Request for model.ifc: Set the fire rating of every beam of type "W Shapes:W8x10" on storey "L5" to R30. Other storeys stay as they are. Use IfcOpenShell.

First a look at what the model holds.

```python
import ifcopenshell
import ifcopenshell.util.element

model = ifcopenshell.open("model.ifc")
print(model.schema)
storey = next(s for s in model.by_type("IfcBuildingStorey") if s.Name == "L5")
beams = [e for e in ifcopenshell.util.element.get_decomposition(storey) if e.is_a("IfcBeam")]
seen = {}
for e in beams:
    element_type = ifcopenshell.util.element.get_type(e)
    key = (element_type.Name if element_type != e and element_type else None, ifcopenshell.util.element.get_pset(e, "Pset_BeamCommon", "FireRating"))
    seen[key] = seen.get(key, 0) + 1
for (name, value), count in sorted(seen.items(), key=str):
    print(count, "x", name, "|", value)
```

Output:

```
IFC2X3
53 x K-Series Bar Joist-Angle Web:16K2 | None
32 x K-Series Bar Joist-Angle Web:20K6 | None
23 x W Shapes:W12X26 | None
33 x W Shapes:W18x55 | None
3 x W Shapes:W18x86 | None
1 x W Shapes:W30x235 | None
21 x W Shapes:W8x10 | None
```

```python
import ifcopenshell
import ifcopenshell.api.pset
import ifcopenshell.util.element

model = ifcopenshell.open("model.ifc")

storey = next(s for s in model.by_type("IfcBuildingStorey") if s.Name == "L5")
beams = [e for e in ifcopenshell.util.element.get_decomposition(storey) if e.is_a("IfcBeam")]

count = 0
for e in beams:
    element_type = ifcopenshell.util.element.get_type(e)
    if element_type in (None, e) or element_type.Name != "W Shapes:W8x10":
        continue
    # add_pset returns the element's existing set when there is one.
    pset = ifcopenshell.api.pset.add_pset(model, product=e, name="Pset_BeamCommon")
    ifcopenshell.api.pset.edit_pset(model, pset=pset, properties={"FireRating": "R30"})
    count += 1

print(count, "beams updated")

model.write("model_updated.ifc")
```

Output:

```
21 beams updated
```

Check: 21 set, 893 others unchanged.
